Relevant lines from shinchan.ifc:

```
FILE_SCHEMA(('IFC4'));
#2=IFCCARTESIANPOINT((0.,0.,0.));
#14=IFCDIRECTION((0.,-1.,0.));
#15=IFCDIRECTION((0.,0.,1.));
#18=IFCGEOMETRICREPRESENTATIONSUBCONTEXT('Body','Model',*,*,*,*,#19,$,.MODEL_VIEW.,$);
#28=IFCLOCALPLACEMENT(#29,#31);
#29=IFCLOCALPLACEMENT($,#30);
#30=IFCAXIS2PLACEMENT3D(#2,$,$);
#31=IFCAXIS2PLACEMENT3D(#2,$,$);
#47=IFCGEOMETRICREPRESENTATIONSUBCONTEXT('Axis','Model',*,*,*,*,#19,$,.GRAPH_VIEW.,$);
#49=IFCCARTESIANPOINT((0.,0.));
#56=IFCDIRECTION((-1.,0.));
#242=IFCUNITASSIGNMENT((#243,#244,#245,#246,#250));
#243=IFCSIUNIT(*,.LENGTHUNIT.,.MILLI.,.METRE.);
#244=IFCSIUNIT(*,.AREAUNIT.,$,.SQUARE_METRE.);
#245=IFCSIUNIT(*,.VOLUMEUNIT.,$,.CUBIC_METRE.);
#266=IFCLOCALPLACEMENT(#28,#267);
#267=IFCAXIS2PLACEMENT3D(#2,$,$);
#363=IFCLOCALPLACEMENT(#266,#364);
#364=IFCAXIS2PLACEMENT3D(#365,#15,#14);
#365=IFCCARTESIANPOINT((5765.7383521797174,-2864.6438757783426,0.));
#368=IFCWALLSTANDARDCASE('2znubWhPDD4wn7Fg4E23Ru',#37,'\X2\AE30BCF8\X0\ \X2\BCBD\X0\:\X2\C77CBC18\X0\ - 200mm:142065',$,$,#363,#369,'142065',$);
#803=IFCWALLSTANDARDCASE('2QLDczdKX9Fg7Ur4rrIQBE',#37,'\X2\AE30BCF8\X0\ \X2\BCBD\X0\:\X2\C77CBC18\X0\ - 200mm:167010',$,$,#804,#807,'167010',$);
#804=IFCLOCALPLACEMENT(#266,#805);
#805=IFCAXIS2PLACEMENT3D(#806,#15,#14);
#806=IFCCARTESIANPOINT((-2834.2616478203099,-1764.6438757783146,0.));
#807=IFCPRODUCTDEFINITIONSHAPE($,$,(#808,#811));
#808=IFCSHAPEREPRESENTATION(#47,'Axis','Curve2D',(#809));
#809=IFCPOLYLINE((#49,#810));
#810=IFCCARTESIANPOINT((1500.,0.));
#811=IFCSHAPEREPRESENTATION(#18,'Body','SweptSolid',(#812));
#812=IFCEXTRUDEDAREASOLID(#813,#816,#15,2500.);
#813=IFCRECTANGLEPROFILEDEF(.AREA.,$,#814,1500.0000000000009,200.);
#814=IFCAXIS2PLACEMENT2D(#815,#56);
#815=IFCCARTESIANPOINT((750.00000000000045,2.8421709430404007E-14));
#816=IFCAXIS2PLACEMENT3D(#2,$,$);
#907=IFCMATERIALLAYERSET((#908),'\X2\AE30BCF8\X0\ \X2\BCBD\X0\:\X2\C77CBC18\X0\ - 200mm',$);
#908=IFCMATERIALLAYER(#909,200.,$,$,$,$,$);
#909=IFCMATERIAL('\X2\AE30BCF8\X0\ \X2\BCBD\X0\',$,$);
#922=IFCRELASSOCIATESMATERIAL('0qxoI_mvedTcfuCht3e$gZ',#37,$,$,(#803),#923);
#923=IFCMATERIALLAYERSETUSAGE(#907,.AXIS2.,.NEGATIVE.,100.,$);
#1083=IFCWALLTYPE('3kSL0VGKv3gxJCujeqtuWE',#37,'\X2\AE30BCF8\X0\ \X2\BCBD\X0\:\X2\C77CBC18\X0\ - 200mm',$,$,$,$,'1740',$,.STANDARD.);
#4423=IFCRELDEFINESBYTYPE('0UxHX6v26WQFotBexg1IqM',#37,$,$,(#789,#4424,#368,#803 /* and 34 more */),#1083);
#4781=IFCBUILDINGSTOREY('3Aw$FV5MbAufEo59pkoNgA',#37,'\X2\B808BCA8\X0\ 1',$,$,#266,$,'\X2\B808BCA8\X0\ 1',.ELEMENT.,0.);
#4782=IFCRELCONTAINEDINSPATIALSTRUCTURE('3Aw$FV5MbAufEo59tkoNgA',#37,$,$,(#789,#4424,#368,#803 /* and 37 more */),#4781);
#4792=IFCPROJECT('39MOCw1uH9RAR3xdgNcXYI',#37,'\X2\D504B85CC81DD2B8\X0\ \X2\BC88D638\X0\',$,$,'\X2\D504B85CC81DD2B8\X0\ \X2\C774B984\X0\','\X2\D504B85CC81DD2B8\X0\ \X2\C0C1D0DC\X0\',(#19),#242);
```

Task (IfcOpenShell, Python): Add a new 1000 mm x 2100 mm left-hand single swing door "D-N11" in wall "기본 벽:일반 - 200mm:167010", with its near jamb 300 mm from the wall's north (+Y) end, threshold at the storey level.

```python
import numpy as np
import ifcopenshell
import ifcopenshell.api.feature
import ifcopenshell.api.geometry
import ifcopenshell.api.root
import ifcopenshell.api.spatial
import ifcopenshell.geom
import ifcopenshell.util.element
import ifcopenshell.util.placement
import ifcopenshell.util.representation
import ifcopenshell.util.shape
import ifcopenshell.util.unit

model = ifcopenshell.open("shinchan.ifc")
unit_scale = ifcopenshell.util.unit.calculate_unit_scale(model)
settings = ifcopenshell.geom.settings()


def volume(element):
    """Net volume in cubic metres, openings subtracted."""
    shape = ifcopenshell.geom.create_shape(settings, element)
    return ifcopenshell.util.shape.get_volume(shape.geometry)


wall = model.by_guid("2QLDczdKX9Fg7Ur4rrIQBE")
storey = ifcopenshell.util.element.get_container(wall, ifc_class="IfcBuildingStorey")
context = ifcopenshell.util.representation.get_context(model, "Model", "Body", "MODEL_VIEW")
before = volume(wall)

width, height, from_end, sill = 1, 2.1, 0.3, 0.0  # metres

# The wall runs along its own X axis, and the end named is its -X end.
wall_shape = ifcopenshell.geom.create_shape(settings, wall)
x, y, z = ifcopenshell.util.shape.get_vertices(wall_shape.geometry).T
start = x.min() + from_end
face, thickness = float(y.min()), float(y.max() - y.min())
wall_matrix = ifcopenshell.util.placement.get_local_placement(wall.ObjectPlacement)
level = ifcopenshell.util.placement.get_local_placement(storey.ObjectPlacement)[2, 3]


def in_wall(x, y):
    """Placement at x, y metres in the wall's axes, at sill height."""
    matrix = wall_matrix.copy()
    matrix[:, 3] = wall_matrix @ np.array([x / unit_scale, y / unit_scale, 0.0, 1.0])
    matrix[2, 3] = level + sill / unit_scale
    return matrix


# Opening: a box that overshoots both wall faces by 50 mm.
opening = ifcopenshell.api.root.create_entity(model, ifc_class="IfcOpeningElement", predefined_type="OPENING")
box = ifcopenshell.api.geometry.add_wall_representation(
    model, context=context, length=width, height=height, thickness=thickness + 0.1
)
ifcopenshell.api.geometry.assign_representation(model, product=opening, representation=box)
ifcopenshell.api.geometry.edit_object_placement(model, product=opening, matrix=in_wall(start, face - 0.05), is_si=False)
ifcopenshell.api.feature.add_feature(model, feature=opening, element=wall)

door = ifcopenshell.api.root.create_entity(model, ifc_class="IfcDoor", name="D-N11", predefined_type="DOOR")
door.OverallWidth, door.OverallHeight = width / unit_scale, height / unit_scale
door.OperationType = "SINGLE_SWING_LEFT"
body = ifcopenshell.api.geometry.add_door_representation(
    model,
    context=context,
    overall_width=door.OverallWidth,
    overall_height=door.OverallHeight,
    operation_type="SINGLE_SWING_LEFT",
    lining_properties={"LiningDepth": thickness / unit_scale, "ThresholdDepth": thickness / unit_scale},
)
ifcopenshell.api.geometry.assign_representation(model, product=door, representation=body)
ifcopenshell.api.spatial.assign_container(model, products=[door], relating_structure=storey)
ifcopenshell.api.feature.add_filling(model, opening=opening, element=door)

# The lining spans the wall, so the door starts at the wall face.
ifcopenshell.api.geometry.edit_object_placement(model, product=door, matrix=in_wall(start, face), is_si=False)

after = volume(wall)

print(f"wall volume {before:.3f} -> {after:.3f} m3")

model.write("shinchan_v2.ifc")
```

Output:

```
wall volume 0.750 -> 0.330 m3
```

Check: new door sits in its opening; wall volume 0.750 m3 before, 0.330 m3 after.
